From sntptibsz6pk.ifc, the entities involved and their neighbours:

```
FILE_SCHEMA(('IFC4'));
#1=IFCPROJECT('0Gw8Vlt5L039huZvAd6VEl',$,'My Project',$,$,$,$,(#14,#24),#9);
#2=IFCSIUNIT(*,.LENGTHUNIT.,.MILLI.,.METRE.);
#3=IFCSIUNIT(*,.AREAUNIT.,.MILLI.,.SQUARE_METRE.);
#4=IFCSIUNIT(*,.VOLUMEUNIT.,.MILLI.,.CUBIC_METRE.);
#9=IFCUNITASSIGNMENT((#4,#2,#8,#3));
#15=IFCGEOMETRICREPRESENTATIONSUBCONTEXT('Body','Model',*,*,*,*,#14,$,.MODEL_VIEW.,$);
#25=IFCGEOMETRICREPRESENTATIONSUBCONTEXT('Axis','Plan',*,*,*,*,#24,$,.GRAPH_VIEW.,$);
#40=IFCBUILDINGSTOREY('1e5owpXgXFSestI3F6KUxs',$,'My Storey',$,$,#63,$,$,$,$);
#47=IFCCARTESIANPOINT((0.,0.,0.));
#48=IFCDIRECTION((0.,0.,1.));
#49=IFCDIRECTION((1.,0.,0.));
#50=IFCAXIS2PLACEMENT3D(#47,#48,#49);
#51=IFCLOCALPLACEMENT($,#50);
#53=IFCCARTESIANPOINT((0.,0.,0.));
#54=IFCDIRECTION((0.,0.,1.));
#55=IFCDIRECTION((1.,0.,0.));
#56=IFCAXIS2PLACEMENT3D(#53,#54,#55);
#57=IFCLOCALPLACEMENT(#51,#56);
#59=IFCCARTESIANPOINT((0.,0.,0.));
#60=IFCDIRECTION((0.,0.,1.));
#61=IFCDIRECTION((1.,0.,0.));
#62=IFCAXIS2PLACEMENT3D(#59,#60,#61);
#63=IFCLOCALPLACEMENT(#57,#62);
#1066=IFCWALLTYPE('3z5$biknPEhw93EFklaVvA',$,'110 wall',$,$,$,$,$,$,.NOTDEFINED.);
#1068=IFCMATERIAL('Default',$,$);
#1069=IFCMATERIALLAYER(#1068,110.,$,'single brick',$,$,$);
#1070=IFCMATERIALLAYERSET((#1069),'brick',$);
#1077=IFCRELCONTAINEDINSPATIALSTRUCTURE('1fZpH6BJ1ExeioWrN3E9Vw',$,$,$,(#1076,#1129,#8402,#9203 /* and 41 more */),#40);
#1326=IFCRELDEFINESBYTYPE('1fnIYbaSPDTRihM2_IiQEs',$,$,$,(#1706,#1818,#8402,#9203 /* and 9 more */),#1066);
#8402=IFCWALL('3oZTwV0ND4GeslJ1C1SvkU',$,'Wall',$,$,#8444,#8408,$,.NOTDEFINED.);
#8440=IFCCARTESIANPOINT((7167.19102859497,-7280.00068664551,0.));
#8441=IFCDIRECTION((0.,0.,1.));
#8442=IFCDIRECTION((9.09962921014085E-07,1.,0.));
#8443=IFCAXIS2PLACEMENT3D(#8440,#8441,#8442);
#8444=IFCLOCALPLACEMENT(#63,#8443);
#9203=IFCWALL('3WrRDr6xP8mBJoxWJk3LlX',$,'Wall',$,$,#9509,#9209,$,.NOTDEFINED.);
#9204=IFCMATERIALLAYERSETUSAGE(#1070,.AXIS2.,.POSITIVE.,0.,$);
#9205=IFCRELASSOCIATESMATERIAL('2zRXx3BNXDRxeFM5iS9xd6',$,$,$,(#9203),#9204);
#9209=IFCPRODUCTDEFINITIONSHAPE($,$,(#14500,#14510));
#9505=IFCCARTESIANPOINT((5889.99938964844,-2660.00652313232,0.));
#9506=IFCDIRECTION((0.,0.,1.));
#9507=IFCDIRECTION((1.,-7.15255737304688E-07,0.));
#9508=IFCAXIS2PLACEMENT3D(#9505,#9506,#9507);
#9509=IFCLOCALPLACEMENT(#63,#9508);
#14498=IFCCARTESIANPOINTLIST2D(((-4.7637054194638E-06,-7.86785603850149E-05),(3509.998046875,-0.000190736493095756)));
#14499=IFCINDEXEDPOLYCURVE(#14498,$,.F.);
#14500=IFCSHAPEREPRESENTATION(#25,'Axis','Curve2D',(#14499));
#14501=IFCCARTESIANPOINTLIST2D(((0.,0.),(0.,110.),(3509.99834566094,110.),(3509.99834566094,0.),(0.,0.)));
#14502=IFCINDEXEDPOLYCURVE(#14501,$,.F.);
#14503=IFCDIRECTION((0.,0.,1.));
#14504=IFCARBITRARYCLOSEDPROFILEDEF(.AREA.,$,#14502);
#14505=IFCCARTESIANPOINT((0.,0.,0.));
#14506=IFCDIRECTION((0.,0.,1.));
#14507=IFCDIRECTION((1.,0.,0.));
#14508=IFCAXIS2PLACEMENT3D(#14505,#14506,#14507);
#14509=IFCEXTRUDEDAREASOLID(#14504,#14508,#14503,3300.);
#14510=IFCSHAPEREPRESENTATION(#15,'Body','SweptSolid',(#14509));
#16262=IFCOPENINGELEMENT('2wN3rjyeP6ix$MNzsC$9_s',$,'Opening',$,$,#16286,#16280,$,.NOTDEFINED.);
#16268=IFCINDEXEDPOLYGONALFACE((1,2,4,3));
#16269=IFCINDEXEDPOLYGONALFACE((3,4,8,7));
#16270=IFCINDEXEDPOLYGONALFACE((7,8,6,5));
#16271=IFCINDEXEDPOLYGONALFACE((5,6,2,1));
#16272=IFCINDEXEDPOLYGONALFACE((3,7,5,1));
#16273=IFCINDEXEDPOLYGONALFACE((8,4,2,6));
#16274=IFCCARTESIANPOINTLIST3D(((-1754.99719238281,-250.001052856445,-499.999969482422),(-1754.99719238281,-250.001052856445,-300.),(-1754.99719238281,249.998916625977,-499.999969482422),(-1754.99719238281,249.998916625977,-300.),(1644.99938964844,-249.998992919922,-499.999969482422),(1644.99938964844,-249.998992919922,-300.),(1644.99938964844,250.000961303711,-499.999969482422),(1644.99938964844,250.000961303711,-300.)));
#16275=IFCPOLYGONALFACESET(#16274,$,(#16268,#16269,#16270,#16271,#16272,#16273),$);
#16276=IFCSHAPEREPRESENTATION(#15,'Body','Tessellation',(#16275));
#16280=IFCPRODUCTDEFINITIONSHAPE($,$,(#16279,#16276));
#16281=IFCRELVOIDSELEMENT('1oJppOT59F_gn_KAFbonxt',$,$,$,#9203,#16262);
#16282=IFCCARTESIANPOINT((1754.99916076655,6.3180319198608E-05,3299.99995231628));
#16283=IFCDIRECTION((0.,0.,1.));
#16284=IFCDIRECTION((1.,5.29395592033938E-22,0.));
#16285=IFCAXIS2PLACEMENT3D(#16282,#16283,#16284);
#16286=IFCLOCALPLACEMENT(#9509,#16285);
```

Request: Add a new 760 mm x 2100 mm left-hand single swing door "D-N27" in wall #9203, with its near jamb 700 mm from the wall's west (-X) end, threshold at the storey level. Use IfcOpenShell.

```python
import numpy as np
import ifcopenshell
import ifcopenshell.api.feature
import ifcopenshell.api.geometry
import ifcopenshell.api.root
import ifcopenshell.api.spatial
import ifcopenshell.geom
import ifcopenshell.util.element
import ifcopenshell.util.placement
import ifcopenshell.util.representation
import ifcopenshell.util.shape
import ifcopenshell.util.unit

model = ifcopenshell.open("sntptibsz6pk.ifc")
unit_scale = ifcopenshell.util.unit.calculate_unit_scale(model)
settings = ifcopenshell.geom.settings()


def volume(element):
    """Net volume in cubic metres, openings subtracted."""
    shape = ifcopenshell.geom.create_shape(settings, element)
    return ifcopenshell.util.shape.get_volume(shape.geometry)


wall = model.by_guid("3WrRDr6xP8mBJoxWJk3LlX")
storey = ifcopenshell.util.element.get_container(wall, ifc_class="IfcBuildingStorey")
context = ifcopenshell.util.representation.get_context(model, "Model", "Body", "MODEL_VIEW")
before = volume(wall)

width, height, from_end, sill = 0.76, 2.1, 0.7, 0.0  # metres

# The wall runs along its own X axis, and the end named is its -X end.
wall_shape = ifcopenshell.geom.create_shape(settings, wall)
x, y, z = ifcopenshell.util.shape.get_vertices(wall_shape.geometry).T
start = x.min() + from_end
face, thickness = float(y.min()), float(y.max() - y.min())
wall_matrix = ifcopenshell.util.placement.get_local_placement(wall.ObjectPlacement)
level = ifcopenshell.util.placement.get_local_placement(storey.ObjectPlacement)[2, 3]


def in_wall(x, y):
    """Placement at x, y metres in the wall's axes, at sill height."""
    matrix = wall_matrix.copy()
    matrix[:, 3] = wall_matrix @ np.array([x / unit_scale, y / unit_scale, 0.0, 1.0])
    matrix[2, 3] = level + sill / unit_scale
    return matrix


# Opening: a box that overshoots both wall faces by 50 mm.
opening = ifcopenshell.api.root.create_entity(model, ifc_class="IfcOpeningElement", predefined_type="OPENING")
box = ifcopenshell.api.geometry.add_wall_representation(
    model, context=context, length=width, height=height, thickness=thickness + 0.1
)
ifcopenshell.api.geometry.assign_representation(model, product=opening, representation=box)
ifcopenshell.api.geometry.edit_object_placement(model, product=opening, matrix=in_wall(start, face - 0.05), is_si=False)
ifcopenshell.api.feature.add_feature(model, feature=opening, element=wall)

door = ifcopenshell.api.root.create_entity(model, ifc_class="IfcDoor", name="D-N27", predefined_type="DOOR")
door.OverallWidth, door.OverallHeight = width / unit_scale, height / unit_scale
door.OperationType = "SINGLE_SWING_LEFT"
body = ifcopenshell.api.geometry.add_door_representation(
    model,
    context=context,
    overall_width=door.OverallWidth,
    overall_height=door.OverallHeight,
    operation_type="SINGLE_SWING_LEFT",
    lining_properties={"LiningDepth": thickness / unit_scale, "ThresholdDepth": thickness / unit_scale},
)
ifcopenshell.api.geometry.assign_representation(model, product=door, representation=body)
ifcopenshell.api.spatial.assign_container(model, products=[door], relating_structure=storey)
ifcopenshell.api.feature.add_filling(model, opening=opening, element=door)

# The lining spans the wall, so the door starts at the wall face.
ifcopenshell.api.geometry.edit_object_placement(model, product=door, matrix=in_wall(start, face), is_si=False)

after = volume(wall)

print(f"wall volume {before:.3f} -> {after:.3f} m3")

model.write("sntptibsz6pk_v2.ifc")
```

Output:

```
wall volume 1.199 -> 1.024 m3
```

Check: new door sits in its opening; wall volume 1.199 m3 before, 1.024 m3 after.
